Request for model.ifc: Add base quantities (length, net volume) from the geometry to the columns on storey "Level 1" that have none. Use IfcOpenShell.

First a look at what the model holds.

```python
import ifcopenshell
import ifcopenshell.util.element
import ifcopenshell.util.unit

model = ifcopenshell.open("model.ifc")
print(model.schema)
for unit_type in ("LENGTHUNIT", "AREAUNIT", "VOLUMEUNIT"):
    print(unit_type, ifcopenshell.util.unit.calculate_unit_scale(model, unit_type))
storey = next(s for s in model.by_type("IfcBuildingStorey") if s.Name == "Level 1")
columns = [e for e in ifcopenshell.util.element.get_decomposition(storey) if e.is_a("IfcColumn")]
for e in sorted(columns, key=lambda e: e.id()):
    print(e.id(), e.is_a(), e.Name, list(ifcopenshell.util.element.get_psets(e, qtos_only=True)), sep=" | ")
```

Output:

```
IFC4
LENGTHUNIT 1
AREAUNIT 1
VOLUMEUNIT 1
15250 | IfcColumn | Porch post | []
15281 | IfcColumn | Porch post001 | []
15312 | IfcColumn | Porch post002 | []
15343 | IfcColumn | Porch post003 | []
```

```python
import ifcopenshell
import ifcopenshell.api.pset
import ifcopenshell.geom
import ifcopenshell.util.element
import ifcopenshell.util.shape
import ifcopenshell.util.unit

model = ifcopenshell.open("model.ifc")
unit_scale = ifcopenshell.util.unit.calculate_unit_scale(model)
volume_scale = ifcopenshell.util.unit.calculate_unit_scale(model, "VOLUMEUNIT")
settings = ifcopenshell.geom.settings()

storey = next(s for s in model.by_type("IfcBuildingStorey") if s.Name == "Level 1")
columns = [e for e in ifcopenshell.util.element.get_decomposition(storey) if e.is_a("IfcColumn")]

for e in sorted(columns, key=lambda e: e.id()):
    if ifcopenshell.util.element.get_psets(e, qtos_only=True, should_inherit=False):
        continue
    # Geometry comes back in metres, in the element's own axes.
    shape = ifcopenshell.geom.create_shape(settings, e)
    values = {
        "Length": ifcopenshell.util.shape.get_z(shape.geometry) / unit_scale,
        "NetVolume": ifcopenshell.util.shape.get_volume(shape.geometry) / volume_scale,
    }
    qto = ifcopenshell.api.pset.add_qto(model, product=e, name="Qto_ColumnBaseQuantities")
    ifcopenshell.api.pset.edit_qto(model, qto=qto, properties=values)
    print(e.id(), {k: round(v, 3) for k, v in values.items()})

model.write("model_edited.ifc")
```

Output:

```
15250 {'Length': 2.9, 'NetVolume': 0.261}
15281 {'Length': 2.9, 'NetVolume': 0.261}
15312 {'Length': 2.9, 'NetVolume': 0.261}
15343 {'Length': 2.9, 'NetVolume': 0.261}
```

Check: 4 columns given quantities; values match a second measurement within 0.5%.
